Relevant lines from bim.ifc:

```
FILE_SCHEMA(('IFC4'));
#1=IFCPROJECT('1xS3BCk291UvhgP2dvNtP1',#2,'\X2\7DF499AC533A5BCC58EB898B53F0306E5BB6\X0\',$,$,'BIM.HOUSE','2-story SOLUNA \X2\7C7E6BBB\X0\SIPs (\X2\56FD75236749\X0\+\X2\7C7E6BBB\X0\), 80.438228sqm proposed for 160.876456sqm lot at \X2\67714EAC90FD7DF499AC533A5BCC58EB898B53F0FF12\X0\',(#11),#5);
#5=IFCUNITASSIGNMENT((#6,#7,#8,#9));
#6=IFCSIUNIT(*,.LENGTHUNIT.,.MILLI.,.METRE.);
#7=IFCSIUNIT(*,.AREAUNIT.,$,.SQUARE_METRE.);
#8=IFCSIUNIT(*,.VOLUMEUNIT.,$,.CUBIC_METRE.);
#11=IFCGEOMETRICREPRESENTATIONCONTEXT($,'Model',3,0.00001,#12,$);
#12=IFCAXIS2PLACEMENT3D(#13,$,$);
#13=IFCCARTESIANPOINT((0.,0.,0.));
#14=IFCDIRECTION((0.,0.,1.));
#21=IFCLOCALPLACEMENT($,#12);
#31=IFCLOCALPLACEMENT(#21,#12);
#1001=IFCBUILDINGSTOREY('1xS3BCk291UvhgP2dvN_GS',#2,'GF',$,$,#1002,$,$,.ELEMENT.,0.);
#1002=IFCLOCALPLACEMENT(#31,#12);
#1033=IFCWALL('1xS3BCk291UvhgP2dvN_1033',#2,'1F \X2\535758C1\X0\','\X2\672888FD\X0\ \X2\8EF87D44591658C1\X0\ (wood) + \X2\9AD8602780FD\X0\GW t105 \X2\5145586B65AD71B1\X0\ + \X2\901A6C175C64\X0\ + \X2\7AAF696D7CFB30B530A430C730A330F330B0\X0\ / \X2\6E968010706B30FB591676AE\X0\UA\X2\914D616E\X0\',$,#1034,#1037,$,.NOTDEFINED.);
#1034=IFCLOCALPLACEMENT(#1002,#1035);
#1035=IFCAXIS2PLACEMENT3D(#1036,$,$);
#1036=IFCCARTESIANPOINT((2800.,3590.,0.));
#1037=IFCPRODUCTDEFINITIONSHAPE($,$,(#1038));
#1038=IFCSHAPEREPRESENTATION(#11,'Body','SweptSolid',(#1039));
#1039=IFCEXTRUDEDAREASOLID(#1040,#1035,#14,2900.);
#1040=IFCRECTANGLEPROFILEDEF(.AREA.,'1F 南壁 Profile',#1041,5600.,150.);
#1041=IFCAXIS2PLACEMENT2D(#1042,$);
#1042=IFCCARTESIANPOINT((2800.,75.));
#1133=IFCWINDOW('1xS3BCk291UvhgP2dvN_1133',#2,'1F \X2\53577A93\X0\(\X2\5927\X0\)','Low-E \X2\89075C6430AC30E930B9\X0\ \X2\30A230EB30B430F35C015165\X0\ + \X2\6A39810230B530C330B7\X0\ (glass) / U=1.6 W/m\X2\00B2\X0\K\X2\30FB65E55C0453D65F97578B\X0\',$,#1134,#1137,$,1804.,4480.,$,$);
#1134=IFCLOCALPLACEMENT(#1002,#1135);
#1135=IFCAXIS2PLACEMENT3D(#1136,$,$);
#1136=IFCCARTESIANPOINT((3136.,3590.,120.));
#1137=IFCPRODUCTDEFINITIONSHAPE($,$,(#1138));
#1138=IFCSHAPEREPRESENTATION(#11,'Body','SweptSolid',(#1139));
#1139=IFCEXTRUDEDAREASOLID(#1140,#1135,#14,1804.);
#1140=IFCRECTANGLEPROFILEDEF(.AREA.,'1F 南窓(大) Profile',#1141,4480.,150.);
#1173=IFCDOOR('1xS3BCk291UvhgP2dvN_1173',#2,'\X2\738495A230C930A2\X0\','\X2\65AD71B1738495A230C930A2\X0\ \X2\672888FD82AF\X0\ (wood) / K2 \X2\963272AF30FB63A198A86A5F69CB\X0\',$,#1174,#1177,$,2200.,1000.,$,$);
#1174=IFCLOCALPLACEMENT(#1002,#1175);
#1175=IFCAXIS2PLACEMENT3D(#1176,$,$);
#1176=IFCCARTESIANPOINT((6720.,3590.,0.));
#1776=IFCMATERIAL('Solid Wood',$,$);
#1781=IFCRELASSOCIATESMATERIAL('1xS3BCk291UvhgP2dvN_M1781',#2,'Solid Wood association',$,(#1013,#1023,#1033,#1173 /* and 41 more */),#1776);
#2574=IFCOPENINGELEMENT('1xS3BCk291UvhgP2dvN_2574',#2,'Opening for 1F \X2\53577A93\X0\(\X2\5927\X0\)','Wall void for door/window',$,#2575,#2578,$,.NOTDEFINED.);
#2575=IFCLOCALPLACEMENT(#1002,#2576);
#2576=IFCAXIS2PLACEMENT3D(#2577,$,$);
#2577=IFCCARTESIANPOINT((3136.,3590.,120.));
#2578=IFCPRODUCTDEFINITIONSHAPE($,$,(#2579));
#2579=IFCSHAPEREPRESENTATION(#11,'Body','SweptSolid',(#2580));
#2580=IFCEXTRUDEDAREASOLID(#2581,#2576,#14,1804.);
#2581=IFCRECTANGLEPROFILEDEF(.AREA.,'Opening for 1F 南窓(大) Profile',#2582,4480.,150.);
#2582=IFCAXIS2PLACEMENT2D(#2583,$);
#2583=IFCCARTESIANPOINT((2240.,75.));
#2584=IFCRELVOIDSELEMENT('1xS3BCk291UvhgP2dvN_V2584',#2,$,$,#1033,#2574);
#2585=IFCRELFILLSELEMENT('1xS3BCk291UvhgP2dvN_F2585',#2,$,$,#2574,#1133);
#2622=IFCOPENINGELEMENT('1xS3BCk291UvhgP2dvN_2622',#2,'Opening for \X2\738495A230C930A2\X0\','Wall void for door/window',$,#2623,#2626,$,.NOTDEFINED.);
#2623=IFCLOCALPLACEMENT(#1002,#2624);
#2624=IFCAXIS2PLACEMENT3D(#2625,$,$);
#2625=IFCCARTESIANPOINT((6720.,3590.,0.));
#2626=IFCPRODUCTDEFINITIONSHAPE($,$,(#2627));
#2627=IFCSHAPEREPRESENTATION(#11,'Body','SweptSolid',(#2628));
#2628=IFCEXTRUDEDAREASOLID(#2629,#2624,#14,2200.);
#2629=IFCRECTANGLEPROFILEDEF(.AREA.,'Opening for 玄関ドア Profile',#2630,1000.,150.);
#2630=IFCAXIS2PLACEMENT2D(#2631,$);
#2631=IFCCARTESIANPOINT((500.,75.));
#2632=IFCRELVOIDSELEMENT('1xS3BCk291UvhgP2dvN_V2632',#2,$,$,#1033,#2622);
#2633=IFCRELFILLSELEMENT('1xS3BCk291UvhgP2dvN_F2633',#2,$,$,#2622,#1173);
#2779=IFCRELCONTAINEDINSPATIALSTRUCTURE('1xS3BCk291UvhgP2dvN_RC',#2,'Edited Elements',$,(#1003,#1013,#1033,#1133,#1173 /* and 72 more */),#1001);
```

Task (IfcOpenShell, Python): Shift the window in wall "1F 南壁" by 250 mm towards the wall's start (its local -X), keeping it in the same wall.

```python
import ifcopenshell
import ifcopenshell.api.geometry
import ifcopenshell.util.placement
import ifcopenshell.util.unit

model = ifcopenshell.open("bim.ifc")
unit_scale = ifcopenshell.util.unit.calculate_unit_scale(model)

window = model.by_guid("1xS3BCk291UvhgP2dvN_1133")
opening = window.FillsVoids[0].RelatingOpeningElement
wall = opening.VoidsElements[0].RelatingBuildingElement

wall_matrix = ifcopenshell.util.placement.get_local_placement(wall.ObjectPlacement)
shift = wall_matrix[:3, 0] * -0.25 / unit_scale
before = ifcopenshell.util.placement.get_local_placement(window.ObjectPlacement)[:3, 3].copy()

# The window is not placed relative to its opening, so move both.
for product in (opening, window):
    matrix = ifcopenshell.util.placement.get_local_placement(product.ObjectPlacement)
    matrix[:3, 3] += shift
    ifcopenshell.api.geometry.edit_object_placement(model, product=product, matrix=matrix, is_si=False)

after = ifcopenshell.util.placement.get_local_placement(window.ObjectPlacement)[:3, 3]
print("window moved by", (after - before).round(3) + 0.0)

model.write("bim_edited.ifc")
```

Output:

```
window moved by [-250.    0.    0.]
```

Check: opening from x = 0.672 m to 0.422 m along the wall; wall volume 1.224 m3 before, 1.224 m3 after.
